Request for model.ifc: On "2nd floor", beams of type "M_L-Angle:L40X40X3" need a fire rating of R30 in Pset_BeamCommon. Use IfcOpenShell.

First a look at what the model holds.

```python
import ifcopenshell
import ifcopenshell.util.element

model = ifcopenshell.open("model.ifc")
print(model.schema)
storey = next(s for s in model.by_type("IfcBuildingStorey") if s.Name == "2nd floor")
beams = [e for e in ifcopenshell.util.element.get_decomposition(storey) if e.is_a("IfcBeam")]
seen = {}
for e in beams:
    element_type = ifcopenshell.util.element.get_type(e)
    key = (element_type.Name if element_type != e and element_type else None, ifcopenshell.util.element.get_pset(e, "Pset_BeamCommon", "FireRating"))
    seen[key] = seen.get(key, 0) + 1
for (name, value), count in sorted(seen.items(), key=str):
    print(count, "x", name, "|", value)
```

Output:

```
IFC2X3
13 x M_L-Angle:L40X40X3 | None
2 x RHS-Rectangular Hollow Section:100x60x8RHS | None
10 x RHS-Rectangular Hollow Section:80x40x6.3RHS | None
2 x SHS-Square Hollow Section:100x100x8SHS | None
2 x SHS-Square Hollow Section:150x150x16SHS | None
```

```python
import ifcopenshell
import ifcopenshell.api.pset
import ifcopenshell.util.element

model = ifcopenshell.open("model.ifc")

storey = next(s for s in model.by_type("IfcBuildingStorey") if s.Name == "2nd floor")
beams = [e for e in ifcopenshell.util.element.get_decomposition(storey) if e.is_a("IfcBeam")]

count = 0
for e in beams:
    element_type = ifcopenshell.util.element.get_type(e)
    if element_type in (None, e) or element_type.Name != "M_L-Angle:L40X40X3":
        continue
    # add_pset returns the element's existing set when there is one.
    pset = ifcopenshell.api.pset.add_pset(model, product=e, name="Pset_BeamCommon")
    ifcopenshell.api.pset.edit_pset(model, pset=pset, properties={"FireRating": "R30"})
    count += 1

print(count, "beams updated")

model.write("model_updated.ifc")
```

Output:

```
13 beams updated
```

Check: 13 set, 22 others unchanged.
